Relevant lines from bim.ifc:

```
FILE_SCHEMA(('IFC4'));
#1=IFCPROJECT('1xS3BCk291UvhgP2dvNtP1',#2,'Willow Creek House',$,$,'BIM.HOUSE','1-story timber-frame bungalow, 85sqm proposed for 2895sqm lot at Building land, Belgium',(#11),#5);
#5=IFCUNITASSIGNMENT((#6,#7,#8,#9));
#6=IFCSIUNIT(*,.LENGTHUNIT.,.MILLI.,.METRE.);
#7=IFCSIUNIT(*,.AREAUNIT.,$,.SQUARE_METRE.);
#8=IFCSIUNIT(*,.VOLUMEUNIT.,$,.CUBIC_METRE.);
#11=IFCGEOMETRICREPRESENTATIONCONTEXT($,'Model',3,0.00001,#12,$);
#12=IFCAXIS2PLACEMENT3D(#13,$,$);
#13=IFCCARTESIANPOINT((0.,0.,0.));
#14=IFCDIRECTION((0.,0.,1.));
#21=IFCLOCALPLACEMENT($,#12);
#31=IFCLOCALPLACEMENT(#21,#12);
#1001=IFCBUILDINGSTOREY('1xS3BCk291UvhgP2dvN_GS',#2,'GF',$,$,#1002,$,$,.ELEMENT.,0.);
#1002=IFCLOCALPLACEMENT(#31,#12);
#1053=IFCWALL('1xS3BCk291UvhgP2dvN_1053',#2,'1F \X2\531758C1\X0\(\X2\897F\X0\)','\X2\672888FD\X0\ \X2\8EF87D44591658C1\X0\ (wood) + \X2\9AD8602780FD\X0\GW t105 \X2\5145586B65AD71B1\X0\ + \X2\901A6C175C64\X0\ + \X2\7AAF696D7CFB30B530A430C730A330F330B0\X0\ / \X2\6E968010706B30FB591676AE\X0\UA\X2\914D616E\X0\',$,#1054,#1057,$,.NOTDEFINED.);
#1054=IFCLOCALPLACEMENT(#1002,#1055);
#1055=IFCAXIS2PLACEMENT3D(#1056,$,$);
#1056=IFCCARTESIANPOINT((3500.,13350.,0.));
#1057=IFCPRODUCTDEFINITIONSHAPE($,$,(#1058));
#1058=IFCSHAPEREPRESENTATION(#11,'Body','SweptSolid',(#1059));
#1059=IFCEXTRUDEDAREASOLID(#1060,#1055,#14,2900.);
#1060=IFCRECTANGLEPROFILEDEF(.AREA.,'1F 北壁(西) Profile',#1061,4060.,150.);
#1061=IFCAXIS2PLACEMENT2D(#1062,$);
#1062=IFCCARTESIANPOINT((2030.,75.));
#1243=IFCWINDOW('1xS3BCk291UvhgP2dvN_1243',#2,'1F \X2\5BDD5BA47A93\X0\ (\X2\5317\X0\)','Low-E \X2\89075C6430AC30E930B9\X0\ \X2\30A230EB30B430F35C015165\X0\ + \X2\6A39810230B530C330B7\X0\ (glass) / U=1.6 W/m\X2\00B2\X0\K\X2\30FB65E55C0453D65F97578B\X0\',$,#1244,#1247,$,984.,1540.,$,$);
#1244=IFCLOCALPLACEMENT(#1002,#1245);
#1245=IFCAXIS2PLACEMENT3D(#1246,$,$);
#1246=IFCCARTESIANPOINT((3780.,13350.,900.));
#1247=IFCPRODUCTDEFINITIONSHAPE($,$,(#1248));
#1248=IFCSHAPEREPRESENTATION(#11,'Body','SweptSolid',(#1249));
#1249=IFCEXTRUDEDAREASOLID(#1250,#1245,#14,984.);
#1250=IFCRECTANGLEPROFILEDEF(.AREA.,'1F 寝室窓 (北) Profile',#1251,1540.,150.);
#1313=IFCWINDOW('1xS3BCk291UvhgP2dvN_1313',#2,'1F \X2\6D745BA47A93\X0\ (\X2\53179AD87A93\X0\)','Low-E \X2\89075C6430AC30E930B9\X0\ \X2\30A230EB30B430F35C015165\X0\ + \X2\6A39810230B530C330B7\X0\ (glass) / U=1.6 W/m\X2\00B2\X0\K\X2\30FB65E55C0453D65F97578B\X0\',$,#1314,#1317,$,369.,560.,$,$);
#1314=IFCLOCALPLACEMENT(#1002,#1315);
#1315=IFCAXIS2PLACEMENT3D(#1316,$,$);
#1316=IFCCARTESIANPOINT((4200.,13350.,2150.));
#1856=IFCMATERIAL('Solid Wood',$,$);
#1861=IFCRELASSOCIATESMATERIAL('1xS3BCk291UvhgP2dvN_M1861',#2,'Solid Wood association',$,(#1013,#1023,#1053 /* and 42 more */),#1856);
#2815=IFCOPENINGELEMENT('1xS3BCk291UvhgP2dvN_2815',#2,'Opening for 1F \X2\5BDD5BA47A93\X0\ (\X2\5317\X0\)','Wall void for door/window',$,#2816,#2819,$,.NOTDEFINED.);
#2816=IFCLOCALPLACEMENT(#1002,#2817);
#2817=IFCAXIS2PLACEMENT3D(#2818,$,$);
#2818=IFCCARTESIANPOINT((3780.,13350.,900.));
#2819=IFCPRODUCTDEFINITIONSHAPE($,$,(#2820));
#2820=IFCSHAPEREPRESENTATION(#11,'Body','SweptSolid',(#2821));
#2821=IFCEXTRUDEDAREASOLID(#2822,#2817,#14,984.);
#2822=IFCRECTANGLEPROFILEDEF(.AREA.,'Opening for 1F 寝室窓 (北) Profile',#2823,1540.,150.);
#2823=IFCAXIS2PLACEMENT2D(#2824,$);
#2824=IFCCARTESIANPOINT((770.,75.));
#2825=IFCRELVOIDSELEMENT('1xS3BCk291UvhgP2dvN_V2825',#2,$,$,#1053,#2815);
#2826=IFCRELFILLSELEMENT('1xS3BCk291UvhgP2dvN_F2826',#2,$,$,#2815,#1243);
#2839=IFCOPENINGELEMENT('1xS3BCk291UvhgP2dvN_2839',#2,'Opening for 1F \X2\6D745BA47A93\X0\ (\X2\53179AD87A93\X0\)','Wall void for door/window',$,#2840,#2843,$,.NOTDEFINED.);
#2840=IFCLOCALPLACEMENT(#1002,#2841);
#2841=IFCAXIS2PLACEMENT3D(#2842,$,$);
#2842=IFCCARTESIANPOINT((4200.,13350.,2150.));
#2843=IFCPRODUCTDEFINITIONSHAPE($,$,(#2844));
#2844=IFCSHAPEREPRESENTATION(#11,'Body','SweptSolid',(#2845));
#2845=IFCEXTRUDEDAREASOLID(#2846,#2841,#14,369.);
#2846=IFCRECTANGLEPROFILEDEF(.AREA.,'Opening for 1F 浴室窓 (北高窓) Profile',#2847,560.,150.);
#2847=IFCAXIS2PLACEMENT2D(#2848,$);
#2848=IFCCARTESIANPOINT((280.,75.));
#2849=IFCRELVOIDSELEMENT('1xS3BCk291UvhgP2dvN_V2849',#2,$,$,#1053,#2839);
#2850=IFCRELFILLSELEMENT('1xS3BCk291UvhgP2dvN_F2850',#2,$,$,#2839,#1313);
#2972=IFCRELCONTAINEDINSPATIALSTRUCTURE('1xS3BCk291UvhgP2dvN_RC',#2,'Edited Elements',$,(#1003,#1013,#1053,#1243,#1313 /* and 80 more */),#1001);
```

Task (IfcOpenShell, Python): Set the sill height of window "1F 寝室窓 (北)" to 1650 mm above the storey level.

```python
import numpy as np
import ifcopenshell
import ifcopenshell.api.geometry
import ifcopenshell.geom
import ifcopenshell.util.element
import ifcopenshell.util.placement
import ifcopenshell.util.shape
import ifcopenshell.util.unit

model = ifcopenshell.open("bim.ifc")
unit_scale = ifcopenshell.util.unit.calculate_unit_scale(model)

window = model.by_id(1243)
opening = window.FillsVoids[0].RelatingOpeningElement
storey = ifcopenshell.util.element.get_container(window, ifc_class="IfcBuildingStorey")
level = ifcopenshell.util.placement.get_local_placement(storey.ObjectPlacement)[2, 3]

# The opening's origin need not be at the sill, so measure its lowest point.
shape = ifcopenshell.geom.create_shape(ifcopenshell.geom.settings(), opening)
bottom = ifcopenshell.util.shape.get_shape_bottom_elevation(shape, shape.geometry) / unit_scale
dz = level + 1.65 / unit_scale - bottom

shift = np.array([0.0, 0.0, dz])
# The window is not placed relative to its opening, so move both.
for product in (opening, window):
    matrix = ifcopenshell.util.placement.get_local_placement(product.ObjectPlacement)
    matrix[:3, 3] += shift
    ifcopenshell.api.geometry.edit_object_placement(model, product=product, matrix=matrix, is_si=False)

print(f"moved by {dz * unit_scale:+.3f} m")

model.write("bim-out.ifc")
```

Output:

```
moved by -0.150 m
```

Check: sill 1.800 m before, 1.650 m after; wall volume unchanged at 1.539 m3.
